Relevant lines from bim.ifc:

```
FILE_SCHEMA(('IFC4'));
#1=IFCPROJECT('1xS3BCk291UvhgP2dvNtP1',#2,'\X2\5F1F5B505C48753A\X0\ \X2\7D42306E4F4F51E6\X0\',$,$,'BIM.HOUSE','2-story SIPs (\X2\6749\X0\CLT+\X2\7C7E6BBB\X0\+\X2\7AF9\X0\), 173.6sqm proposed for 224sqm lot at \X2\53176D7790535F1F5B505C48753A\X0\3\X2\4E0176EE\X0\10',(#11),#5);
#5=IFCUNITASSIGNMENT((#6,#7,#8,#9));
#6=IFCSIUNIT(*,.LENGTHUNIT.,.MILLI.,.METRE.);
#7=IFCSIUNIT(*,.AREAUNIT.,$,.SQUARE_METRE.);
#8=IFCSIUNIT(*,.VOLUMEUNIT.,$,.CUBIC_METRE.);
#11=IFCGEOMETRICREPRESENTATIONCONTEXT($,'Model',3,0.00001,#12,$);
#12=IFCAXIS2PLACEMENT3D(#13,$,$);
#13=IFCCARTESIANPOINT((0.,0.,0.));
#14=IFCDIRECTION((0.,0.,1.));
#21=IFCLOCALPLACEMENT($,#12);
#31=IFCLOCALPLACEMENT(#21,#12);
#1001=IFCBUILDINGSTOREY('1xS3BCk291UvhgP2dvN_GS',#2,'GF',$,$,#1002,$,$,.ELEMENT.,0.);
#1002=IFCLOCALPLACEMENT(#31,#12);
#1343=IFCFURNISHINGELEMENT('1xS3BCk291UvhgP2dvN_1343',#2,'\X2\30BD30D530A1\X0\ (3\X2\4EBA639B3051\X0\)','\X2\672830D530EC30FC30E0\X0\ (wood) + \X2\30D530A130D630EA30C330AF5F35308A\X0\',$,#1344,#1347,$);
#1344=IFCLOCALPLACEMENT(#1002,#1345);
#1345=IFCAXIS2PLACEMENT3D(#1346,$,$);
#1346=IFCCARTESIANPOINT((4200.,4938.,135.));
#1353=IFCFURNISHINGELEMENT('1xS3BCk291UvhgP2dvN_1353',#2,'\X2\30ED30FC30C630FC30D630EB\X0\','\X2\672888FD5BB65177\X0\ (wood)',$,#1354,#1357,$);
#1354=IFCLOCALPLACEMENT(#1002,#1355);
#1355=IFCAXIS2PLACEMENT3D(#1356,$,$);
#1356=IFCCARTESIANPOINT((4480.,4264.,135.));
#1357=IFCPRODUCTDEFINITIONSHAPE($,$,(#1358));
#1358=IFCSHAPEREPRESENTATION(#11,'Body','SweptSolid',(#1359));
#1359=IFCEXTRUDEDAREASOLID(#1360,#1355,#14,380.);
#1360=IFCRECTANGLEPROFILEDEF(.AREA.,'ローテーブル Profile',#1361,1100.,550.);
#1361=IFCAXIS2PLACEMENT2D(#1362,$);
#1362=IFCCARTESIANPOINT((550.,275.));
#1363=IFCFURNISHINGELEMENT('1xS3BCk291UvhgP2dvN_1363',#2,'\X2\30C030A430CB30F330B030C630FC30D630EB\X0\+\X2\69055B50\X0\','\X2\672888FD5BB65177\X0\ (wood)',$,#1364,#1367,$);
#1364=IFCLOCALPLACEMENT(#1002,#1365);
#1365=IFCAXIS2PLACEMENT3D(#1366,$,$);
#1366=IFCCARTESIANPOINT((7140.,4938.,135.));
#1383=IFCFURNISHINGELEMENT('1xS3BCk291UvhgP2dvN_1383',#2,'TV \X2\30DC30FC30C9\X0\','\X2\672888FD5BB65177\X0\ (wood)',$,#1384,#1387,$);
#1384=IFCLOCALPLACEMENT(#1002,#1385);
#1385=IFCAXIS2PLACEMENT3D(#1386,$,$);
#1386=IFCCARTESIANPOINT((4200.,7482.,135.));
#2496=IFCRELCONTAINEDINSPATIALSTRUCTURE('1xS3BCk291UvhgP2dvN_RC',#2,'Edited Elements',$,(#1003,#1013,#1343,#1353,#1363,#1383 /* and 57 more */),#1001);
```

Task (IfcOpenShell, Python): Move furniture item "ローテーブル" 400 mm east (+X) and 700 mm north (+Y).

```python
import ifcopenshell
import ifcopenshell.api.geometry
import ifcopenshell.util.placement
import ifcopenshell.util.unit

model = ifcopenshell.open("bim.ifc")
unit_scale = ifcopenshell.util.unit.calculate_unit_scale(model)

item = model.by_guid("1xS3BCk291UvhgP2dvN_1353")
matrix = ifcopenshell.util.placement.get_local_placement(item.ObjectPlacement)
matrix[0, 3] += 0.4 / unit_scale
matrix[1, 3] += 0.7 / unit_scale
ifcopenshell.api.geometry.edit_object_placement(model, product=item, matrix=matrix, is_si=False)

print(ifcopenshell.util.placement.get_local_placement(item.ObjectPlacement).round(3) + 0.0)

model.write("bim_rev.ifc")
```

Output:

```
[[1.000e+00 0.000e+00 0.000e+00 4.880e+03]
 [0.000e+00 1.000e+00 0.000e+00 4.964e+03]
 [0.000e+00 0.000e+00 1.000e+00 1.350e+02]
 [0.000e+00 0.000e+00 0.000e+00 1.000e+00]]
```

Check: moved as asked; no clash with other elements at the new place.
